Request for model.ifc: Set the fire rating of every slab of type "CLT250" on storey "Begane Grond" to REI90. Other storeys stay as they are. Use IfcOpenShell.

First a look at what the model holds.

```python
import ifcopenshell
import ifcopenshell.util.element

model = ifcopenshell.open("model.ifc")
print(model.schema)
storey = next(s for s in model.by_type("IfcBuildingStorey") if s.Name == "Begane Grond")
slabs = [e for e in ifcopenshell.util.element.get_decomposition(storey) if e.is_a("IfcSlab")]
seen = {}
for e in slabs:
    element_type = ifcopenshell.util.element.get_type(e)
    key = (element_type.Name if element_type != e and element_type else None, ifcopenshell.util.element.get_pset(e, "Pset_SlabCommon", "FireRating"))
    seen[key] = seen.get(key, 0) + 1
for (name, value), count in sorted(seen.items(), key=str):
    print(count, "x", name, "|", value)
```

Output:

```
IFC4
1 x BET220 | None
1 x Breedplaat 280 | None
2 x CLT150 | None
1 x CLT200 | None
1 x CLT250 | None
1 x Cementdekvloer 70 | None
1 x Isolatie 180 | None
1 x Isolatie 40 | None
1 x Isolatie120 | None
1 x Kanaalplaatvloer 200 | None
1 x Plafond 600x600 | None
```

```python
import ifcopenshell
import ifcopenshell.api.pset
import ifcopenshell.util.element

model = ifcopenshell.open("model.ifc")

storey = next(s for s in model.by_type("IfcBuildingStorey") if s.Name == "Begane Grond")
slabs = [e for e in ifcopenshell.util.element.get_decomposition(storey) if e.is_a("IfcSlab")]

count = 0
for e in slabs:
    element_type = ifcopenshell.util.element.get_type(e)
    if element_type in (None, e) or element_type.Name != "CLT250":
        continue
    # add_pset returns the element's existing set when there is one.
    pset = ifcopenshell.api.pset.add_pset(model, product=e, name="Pset_SlabCommon")
    ifcopenshell.api.pset.edit_pset(model, pset=pset, properties={"FireRating": "REI90"})
    count += 1

print(count, "slabs updated")

model.write("model_v2.ifc")
```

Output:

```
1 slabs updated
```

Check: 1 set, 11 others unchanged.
